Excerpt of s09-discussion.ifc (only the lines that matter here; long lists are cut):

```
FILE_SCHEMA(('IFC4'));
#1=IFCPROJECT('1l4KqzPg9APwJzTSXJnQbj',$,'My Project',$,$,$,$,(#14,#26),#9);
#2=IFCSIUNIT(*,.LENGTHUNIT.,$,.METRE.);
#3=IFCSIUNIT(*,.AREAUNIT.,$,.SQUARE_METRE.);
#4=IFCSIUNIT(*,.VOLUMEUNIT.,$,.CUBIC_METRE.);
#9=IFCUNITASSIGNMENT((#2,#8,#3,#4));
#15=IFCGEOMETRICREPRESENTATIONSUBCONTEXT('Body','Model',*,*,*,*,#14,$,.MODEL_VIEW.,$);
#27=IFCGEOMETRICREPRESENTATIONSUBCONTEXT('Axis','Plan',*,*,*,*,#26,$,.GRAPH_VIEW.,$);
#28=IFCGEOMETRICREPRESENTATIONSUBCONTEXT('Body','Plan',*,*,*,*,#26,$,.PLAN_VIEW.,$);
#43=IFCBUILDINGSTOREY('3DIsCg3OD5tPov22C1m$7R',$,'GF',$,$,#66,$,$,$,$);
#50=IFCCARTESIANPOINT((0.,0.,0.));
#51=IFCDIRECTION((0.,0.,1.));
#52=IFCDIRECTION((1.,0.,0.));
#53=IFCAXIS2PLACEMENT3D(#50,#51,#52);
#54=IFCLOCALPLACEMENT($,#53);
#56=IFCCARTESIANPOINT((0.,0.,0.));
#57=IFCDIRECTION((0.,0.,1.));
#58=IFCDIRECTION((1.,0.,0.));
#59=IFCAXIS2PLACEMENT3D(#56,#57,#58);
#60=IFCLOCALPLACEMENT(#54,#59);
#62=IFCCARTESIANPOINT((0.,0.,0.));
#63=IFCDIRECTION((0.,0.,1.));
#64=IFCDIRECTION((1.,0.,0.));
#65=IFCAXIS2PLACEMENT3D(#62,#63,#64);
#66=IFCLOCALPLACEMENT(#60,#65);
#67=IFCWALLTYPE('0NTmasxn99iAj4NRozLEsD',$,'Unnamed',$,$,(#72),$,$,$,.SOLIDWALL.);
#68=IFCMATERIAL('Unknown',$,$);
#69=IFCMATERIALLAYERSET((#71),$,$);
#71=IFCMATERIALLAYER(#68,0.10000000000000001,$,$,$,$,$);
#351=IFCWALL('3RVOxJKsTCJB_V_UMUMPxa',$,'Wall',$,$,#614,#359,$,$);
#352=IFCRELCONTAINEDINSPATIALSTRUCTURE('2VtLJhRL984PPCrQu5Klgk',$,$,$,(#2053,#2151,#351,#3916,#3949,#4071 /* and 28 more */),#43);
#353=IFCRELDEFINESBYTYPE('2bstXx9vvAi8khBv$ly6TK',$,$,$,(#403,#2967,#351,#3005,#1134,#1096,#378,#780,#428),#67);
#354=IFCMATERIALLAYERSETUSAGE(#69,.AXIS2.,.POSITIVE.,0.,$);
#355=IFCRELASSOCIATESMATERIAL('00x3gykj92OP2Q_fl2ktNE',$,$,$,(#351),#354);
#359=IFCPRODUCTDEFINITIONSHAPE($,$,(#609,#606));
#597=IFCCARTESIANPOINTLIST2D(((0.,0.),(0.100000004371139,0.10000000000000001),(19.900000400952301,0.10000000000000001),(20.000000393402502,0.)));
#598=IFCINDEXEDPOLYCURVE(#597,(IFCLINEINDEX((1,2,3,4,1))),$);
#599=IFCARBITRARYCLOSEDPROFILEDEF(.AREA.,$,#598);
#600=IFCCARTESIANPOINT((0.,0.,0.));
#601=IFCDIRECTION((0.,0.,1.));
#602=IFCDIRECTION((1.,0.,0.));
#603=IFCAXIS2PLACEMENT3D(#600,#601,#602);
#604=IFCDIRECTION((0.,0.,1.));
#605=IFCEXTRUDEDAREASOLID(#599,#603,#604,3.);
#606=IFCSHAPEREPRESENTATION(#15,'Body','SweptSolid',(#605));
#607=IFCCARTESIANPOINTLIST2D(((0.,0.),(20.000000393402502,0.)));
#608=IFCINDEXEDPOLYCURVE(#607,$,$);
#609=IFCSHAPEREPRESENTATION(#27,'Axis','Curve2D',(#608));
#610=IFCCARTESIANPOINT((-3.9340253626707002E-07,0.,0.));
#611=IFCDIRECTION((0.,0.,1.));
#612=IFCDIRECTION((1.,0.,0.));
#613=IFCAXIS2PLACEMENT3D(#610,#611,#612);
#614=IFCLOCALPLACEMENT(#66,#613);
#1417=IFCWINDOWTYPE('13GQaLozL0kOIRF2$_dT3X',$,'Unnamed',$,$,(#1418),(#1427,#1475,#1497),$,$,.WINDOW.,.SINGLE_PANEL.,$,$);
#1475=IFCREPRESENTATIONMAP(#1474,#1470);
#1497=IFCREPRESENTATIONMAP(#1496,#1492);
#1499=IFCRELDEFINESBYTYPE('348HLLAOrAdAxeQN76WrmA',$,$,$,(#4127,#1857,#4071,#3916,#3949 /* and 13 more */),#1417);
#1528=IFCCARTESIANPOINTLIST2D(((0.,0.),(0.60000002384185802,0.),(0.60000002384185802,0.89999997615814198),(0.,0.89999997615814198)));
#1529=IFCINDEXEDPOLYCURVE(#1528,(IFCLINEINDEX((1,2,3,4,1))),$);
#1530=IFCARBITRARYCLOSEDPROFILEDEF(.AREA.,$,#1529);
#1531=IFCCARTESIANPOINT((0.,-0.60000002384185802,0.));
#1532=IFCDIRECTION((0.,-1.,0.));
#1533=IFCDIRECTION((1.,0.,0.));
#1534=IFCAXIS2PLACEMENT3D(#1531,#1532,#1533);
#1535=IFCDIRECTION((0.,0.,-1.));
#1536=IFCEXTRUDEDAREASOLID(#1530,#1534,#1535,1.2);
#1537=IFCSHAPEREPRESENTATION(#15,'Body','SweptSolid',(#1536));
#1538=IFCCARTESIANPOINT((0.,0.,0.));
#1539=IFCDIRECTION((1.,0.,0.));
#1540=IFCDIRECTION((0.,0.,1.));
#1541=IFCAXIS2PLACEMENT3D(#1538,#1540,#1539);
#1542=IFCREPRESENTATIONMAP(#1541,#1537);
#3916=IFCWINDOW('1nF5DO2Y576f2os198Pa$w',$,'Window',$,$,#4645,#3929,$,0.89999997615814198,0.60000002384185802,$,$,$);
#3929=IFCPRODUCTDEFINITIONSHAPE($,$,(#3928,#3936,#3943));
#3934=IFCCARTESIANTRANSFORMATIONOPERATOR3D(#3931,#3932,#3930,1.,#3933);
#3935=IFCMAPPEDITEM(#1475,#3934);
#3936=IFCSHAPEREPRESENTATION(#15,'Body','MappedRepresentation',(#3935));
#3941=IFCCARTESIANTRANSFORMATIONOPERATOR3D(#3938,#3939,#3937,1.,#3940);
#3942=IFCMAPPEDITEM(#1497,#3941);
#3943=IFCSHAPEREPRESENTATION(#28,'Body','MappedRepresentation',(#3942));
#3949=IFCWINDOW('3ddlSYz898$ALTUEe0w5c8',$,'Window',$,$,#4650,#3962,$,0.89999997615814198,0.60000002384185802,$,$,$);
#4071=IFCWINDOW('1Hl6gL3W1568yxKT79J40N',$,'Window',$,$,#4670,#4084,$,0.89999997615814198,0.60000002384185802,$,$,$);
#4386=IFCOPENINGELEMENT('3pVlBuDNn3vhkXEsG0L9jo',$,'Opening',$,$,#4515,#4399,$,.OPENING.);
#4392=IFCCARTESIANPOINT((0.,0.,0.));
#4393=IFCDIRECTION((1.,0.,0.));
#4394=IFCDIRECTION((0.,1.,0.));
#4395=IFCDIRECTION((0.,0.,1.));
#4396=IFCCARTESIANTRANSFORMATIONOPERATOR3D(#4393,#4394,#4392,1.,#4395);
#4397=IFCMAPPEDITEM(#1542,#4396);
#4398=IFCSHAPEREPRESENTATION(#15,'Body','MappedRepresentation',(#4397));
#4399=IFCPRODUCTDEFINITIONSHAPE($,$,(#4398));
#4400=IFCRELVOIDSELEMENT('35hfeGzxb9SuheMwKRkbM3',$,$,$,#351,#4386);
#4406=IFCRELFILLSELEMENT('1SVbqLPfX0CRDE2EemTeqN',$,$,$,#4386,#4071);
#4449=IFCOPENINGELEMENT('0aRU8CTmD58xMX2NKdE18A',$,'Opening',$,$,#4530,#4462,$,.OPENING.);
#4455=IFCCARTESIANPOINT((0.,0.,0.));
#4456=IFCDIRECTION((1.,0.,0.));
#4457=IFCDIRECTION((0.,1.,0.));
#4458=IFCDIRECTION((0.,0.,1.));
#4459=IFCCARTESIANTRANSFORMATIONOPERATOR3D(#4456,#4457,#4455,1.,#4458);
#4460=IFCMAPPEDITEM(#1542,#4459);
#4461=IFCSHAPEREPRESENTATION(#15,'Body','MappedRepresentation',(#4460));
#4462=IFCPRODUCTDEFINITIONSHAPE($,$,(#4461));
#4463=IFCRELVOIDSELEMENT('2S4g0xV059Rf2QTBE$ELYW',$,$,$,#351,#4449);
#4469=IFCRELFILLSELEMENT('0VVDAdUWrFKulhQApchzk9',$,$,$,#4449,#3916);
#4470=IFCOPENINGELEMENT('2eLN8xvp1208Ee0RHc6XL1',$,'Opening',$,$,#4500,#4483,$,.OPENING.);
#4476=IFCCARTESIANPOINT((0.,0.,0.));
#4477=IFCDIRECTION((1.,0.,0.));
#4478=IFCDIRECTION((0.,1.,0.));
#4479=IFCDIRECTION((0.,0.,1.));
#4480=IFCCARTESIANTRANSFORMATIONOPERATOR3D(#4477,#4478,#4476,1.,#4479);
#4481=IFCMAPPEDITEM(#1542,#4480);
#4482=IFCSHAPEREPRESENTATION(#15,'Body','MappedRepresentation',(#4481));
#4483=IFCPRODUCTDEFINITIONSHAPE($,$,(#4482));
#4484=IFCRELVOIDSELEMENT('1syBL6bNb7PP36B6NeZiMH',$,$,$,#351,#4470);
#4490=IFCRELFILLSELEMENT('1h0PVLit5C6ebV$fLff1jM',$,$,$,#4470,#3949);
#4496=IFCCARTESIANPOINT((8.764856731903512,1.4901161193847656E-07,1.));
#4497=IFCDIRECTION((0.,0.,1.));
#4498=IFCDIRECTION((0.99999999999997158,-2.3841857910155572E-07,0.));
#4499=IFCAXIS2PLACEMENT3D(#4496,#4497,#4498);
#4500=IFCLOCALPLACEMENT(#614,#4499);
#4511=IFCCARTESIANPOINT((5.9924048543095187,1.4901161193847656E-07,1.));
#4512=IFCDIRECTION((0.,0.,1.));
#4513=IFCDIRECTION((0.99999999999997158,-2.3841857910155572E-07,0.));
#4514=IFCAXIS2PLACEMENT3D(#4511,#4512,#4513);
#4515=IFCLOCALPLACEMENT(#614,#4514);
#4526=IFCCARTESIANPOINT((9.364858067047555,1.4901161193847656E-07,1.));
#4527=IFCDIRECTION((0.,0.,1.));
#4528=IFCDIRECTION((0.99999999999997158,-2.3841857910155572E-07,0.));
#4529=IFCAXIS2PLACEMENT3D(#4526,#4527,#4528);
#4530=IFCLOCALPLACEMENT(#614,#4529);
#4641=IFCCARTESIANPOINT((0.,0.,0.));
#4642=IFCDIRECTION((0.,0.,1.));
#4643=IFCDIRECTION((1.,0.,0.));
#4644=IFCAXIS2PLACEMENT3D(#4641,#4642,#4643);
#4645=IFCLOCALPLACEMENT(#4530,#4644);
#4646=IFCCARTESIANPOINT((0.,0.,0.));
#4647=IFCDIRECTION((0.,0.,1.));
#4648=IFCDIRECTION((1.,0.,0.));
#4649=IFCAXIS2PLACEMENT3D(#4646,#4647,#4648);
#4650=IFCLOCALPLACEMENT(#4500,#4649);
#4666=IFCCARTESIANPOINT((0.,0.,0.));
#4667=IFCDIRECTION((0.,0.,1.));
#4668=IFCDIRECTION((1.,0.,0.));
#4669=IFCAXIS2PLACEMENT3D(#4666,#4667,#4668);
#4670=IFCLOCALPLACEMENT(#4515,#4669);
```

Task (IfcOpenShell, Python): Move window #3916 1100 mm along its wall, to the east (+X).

```python
import ifcopenshell
import ifcopenshell.api.geometry
import ifcopenshell.util.placement
import ifcopenshell.util.unit

model = ifcopenshell.open("s09-discussion.ifc")
unit_scale = ifcopenshell.util.unit.calculate_unit_scale(model)

window = model.by_guid("1nF5DO2Y576f2os198Pa$w")
opening = window.FillsVoids[0].RelatingOpeningElement
wall = opening.VoidsElements[0].RelatingBuildingElement

wall_matrix = ifcopenshell.util.placement.get_local_placement(wall.ObjectPlacement)
shift = wall_matrix[:3, 0] * 1.1 / unit_scale
before = ifcopenshell.util.placement.get_local_placement(window.ObjectPlacement)[:3, 3].copy()

# The window is placed relative to its opening, so it follows when the opening moves.
matrix = ifcopenshell.util.placement.get_local_placement(opening.ObjectPlacement)
matrix[:3, 3] += shift
ifcopenshell.api.geometry.edit_object_placement(
    model, product=opening, matrix=matrix, is_si=False, should_transform_children=True
)

after = ifcopenshell.util.placement.get_local_placement(window.ObjectPlacement)[:3, 3]
print("window moved by", (after - before).round(3) + 0.0)

model.write("s09-discussion_updated.ifc")
```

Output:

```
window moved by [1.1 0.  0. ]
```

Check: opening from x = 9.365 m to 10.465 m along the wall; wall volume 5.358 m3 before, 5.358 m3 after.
